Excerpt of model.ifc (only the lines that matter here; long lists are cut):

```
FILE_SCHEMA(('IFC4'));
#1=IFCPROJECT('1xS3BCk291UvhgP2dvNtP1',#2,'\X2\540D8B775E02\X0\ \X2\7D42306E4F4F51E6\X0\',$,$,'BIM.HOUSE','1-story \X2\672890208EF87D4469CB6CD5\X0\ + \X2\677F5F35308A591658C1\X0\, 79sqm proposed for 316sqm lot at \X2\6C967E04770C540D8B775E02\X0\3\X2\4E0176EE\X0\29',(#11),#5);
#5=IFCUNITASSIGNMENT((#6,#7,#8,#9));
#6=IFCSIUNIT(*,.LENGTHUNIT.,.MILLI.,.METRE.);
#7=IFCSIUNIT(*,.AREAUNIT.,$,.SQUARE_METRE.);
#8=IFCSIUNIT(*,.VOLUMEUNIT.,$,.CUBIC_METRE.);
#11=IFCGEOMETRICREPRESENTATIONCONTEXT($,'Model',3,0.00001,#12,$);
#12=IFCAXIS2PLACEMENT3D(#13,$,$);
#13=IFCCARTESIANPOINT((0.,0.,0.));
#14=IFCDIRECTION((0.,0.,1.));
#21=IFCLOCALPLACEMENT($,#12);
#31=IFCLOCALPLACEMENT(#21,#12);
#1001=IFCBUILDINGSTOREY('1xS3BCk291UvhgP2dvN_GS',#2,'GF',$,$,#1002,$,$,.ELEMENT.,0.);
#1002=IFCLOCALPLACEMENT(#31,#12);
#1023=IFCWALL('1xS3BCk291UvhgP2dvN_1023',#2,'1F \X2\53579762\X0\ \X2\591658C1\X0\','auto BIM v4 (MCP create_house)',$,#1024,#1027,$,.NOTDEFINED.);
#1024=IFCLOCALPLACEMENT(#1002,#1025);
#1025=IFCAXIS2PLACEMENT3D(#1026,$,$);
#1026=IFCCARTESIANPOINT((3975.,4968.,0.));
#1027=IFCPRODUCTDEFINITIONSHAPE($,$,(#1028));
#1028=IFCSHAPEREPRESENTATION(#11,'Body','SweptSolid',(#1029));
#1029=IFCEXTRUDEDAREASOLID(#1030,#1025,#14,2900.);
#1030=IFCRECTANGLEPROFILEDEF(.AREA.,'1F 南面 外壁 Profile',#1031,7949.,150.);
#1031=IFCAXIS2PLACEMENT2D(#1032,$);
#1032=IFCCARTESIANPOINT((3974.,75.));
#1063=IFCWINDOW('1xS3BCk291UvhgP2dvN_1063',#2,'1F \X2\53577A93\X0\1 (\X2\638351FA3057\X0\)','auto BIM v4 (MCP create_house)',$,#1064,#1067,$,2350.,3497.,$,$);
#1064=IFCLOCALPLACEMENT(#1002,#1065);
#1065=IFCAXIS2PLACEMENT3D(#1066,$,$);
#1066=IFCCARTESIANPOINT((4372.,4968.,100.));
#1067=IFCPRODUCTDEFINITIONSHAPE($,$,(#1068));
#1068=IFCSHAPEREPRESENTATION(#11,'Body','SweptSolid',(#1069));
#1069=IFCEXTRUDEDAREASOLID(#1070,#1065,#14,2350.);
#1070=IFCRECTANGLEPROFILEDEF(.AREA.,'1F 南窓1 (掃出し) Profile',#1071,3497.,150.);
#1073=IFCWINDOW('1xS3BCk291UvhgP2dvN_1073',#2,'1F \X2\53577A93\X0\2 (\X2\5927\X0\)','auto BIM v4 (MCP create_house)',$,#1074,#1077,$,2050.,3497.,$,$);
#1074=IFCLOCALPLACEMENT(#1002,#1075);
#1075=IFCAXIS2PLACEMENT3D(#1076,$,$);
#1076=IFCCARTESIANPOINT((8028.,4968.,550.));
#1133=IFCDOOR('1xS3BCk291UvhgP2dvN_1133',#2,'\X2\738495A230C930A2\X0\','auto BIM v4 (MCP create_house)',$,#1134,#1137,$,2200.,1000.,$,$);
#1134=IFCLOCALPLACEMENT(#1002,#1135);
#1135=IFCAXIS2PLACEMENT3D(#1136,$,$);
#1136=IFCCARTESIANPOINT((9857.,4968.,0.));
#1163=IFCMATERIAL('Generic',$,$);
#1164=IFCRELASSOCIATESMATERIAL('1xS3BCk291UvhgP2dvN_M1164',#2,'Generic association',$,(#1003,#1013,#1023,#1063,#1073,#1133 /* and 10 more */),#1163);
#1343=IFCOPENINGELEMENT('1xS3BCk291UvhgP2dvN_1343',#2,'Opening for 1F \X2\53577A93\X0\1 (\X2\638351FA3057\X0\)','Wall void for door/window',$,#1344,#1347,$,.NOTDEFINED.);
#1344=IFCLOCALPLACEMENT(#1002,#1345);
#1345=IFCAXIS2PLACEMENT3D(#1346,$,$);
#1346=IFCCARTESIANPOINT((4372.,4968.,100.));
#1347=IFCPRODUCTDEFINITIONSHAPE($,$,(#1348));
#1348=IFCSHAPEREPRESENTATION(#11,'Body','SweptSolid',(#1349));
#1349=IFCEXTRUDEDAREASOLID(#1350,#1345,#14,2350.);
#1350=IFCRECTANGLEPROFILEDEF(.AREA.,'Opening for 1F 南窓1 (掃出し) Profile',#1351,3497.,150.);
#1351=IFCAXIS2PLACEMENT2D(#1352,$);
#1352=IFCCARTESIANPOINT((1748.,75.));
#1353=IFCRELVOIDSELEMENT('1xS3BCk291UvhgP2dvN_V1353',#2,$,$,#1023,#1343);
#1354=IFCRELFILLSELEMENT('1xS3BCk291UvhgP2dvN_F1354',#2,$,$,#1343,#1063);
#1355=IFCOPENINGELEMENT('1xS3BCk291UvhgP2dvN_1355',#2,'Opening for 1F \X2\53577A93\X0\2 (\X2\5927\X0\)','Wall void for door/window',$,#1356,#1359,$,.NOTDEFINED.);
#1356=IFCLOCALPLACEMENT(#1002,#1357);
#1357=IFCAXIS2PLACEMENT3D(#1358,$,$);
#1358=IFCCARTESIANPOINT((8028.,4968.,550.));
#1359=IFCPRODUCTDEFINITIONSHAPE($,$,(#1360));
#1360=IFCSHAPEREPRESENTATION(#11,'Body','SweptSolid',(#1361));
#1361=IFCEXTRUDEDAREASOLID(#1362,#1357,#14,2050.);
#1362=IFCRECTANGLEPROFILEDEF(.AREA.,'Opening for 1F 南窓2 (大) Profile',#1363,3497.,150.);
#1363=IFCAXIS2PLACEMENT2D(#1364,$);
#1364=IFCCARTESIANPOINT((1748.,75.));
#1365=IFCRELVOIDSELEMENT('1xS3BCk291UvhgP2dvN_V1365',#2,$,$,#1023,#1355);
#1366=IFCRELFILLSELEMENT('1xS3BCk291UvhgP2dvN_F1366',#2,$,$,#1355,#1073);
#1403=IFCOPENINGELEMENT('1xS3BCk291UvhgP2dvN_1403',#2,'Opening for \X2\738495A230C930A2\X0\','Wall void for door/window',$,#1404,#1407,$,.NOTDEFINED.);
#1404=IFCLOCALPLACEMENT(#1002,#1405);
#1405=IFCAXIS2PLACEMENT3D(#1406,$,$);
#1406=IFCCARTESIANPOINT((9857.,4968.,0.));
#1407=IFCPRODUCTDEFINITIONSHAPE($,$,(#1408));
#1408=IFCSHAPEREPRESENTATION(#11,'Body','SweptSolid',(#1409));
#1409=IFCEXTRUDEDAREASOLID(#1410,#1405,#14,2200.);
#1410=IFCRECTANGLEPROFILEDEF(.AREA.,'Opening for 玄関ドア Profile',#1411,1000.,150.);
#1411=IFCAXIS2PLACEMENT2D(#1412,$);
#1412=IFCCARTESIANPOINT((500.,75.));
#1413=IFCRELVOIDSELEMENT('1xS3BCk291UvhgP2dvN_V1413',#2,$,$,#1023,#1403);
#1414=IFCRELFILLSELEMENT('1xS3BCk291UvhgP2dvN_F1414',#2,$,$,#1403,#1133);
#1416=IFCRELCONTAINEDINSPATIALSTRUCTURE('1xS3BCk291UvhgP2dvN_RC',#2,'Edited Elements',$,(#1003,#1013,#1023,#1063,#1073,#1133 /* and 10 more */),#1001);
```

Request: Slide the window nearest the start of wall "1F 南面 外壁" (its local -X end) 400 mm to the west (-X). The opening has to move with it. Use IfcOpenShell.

```python
import ifcopenshell
import ifcopenshell.api.geometry
import ifcopenshell.util.placement
import ifcopenshell.util.unit

model = ifcopenshell.open("model.ifc")
unit_scale = ifcopenshell.util.unit.calculate_unit_scale(model)

window = model.by_guid("1xS3BCk291UvhgP2dvN_1063")
opening = window.FillsVoids[0].RelatingOpeningElement
wall = opening.VoidsElements[0].RelatingBuildingElement

wall_matrix = ifcopenshell.util.placement.get_local_placement(wall.ObjectPlacement)
shift = wall_matrix[:3, 0] * -0.4 / unit_scale
before = ifcopenshell.util.placement.get_local_placement(window.ObjectPlacement)[:3, 3].copy()

# The window is not placed relative to its opening, so move both.
for product in (opening, window):
    matrix = ifcopenshell.util.placement.get_local_placement(product.ObjectPlacement)
    matrix[:3, 3] += shift
    ifcopenshell.api.geometry.edit_object_placement(model, product=product, matrix=matrix, is_si=False)

after = ifcopenshell.util.placement.get_local_placement(window.ObjectPlacement)[:3, 3]
print("window moved by", (after - before).round(3) + 0.0)

model.write("model_rev.ifc")
```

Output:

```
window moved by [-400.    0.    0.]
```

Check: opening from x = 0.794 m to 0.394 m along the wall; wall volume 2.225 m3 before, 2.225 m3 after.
